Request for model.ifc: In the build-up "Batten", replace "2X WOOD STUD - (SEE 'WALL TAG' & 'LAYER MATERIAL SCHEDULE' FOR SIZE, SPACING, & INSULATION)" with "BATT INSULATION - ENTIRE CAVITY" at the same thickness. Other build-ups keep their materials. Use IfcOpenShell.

First a look at what the model holds.

```python
import ifcopenshell
import ifcopenshell.util.element

model = ifcopenshell.open("model.ifc")
print(model.schema)
for layer_set in model.by_type("IfcMaterialLayerSet"):
    if layer_set.LayerSetName == "Batten":
        for layer in layer_set.MaterialLayers:
            print(layer.id(), layer.Material and layer.Material.Name, layer.LayerThickness, sep=" | ")
        print(len(ifcopenshell.util.element.get_elements_by_material(model, layer_set)), "elements and types use it")
print(sorted(m.Name for m in model.by_type("IfcMaterial") if m.Name)[:60])
```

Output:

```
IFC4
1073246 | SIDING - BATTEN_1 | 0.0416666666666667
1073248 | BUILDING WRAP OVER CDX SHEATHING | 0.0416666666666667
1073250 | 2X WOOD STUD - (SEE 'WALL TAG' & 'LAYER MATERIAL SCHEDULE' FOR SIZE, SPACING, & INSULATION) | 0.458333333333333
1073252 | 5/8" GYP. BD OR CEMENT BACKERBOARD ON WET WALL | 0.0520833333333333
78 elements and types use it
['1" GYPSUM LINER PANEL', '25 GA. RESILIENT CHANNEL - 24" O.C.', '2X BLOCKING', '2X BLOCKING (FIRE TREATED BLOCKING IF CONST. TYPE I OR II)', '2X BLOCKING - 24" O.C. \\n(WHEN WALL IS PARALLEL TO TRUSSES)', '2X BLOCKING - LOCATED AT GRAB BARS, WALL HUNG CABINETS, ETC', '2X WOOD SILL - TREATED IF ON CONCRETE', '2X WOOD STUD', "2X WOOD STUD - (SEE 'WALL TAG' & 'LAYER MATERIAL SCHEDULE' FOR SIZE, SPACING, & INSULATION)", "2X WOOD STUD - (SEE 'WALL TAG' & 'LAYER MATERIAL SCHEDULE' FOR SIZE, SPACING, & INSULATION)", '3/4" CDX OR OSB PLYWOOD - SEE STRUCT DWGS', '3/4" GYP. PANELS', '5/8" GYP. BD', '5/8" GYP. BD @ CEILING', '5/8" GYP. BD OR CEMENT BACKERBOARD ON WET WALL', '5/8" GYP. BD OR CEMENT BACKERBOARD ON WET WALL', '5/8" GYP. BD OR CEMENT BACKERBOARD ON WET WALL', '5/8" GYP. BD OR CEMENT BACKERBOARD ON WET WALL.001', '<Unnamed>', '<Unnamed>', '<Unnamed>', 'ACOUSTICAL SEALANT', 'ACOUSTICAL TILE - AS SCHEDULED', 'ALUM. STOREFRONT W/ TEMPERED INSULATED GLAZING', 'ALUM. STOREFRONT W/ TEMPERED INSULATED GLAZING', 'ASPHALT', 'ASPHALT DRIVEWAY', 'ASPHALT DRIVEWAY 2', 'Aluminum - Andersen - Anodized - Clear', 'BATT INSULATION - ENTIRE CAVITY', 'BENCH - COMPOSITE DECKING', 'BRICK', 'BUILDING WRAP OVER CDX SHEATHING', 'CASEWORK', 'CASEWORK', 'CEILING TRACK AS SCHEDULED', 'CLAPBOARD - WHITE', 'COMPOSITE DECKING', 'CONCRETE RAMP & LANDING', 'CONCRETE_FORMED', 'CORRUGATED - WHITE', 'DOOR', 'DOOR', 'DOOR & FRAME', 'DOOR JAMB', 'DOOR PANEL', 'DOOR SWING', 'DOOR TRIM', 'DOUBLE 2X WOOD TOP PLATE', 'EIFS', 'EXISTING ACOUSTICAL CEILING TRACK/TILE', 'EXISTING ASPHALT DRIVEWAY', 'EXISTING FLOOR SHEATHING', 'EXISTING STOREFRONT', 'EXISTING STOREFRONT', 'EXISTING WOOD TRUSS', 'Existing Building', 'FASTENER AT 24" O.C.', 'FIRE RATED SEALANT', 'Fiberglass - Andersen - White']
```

```python
import ifcopenshell
import ifcopenshell.api.material

model = ifcopenshell.open("model.ifc")

layer_set = next(s for s in model.by_type("IfcMaterialLayerSet") if s.LayerSetName == "Batten")
layer = next(l for l in layer_set.MaterialLayers if l.Material and l.Material.Name == "2X WOOD STUD - (SEE 'WALL TAG' & 'LAYER MATERIAL SCHEDULE' FOR SIZE, SPACING, & INSULATION)")
material = next(m for m in model.by_type("IfcMaterial") if m.Name == "BATT INSULATION - ENTIRE CAVITY")

# Point this one layer at the other material; renaming the old one would change it everywhere.
ifcopenshell.api.material.edit_layer(model, layer=layer, attributes={}, material=material)

print([l.Material.Name if l.Material else None for l in layer_set.MaterialLayers])

model.write("model_v2.ifc")
```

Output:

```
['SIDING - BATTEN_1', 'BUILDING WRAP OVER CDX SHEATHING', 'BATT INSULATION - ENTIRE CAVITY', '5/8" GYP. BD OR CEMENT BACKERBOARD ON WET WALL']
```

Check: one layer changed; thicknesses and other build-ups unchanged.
